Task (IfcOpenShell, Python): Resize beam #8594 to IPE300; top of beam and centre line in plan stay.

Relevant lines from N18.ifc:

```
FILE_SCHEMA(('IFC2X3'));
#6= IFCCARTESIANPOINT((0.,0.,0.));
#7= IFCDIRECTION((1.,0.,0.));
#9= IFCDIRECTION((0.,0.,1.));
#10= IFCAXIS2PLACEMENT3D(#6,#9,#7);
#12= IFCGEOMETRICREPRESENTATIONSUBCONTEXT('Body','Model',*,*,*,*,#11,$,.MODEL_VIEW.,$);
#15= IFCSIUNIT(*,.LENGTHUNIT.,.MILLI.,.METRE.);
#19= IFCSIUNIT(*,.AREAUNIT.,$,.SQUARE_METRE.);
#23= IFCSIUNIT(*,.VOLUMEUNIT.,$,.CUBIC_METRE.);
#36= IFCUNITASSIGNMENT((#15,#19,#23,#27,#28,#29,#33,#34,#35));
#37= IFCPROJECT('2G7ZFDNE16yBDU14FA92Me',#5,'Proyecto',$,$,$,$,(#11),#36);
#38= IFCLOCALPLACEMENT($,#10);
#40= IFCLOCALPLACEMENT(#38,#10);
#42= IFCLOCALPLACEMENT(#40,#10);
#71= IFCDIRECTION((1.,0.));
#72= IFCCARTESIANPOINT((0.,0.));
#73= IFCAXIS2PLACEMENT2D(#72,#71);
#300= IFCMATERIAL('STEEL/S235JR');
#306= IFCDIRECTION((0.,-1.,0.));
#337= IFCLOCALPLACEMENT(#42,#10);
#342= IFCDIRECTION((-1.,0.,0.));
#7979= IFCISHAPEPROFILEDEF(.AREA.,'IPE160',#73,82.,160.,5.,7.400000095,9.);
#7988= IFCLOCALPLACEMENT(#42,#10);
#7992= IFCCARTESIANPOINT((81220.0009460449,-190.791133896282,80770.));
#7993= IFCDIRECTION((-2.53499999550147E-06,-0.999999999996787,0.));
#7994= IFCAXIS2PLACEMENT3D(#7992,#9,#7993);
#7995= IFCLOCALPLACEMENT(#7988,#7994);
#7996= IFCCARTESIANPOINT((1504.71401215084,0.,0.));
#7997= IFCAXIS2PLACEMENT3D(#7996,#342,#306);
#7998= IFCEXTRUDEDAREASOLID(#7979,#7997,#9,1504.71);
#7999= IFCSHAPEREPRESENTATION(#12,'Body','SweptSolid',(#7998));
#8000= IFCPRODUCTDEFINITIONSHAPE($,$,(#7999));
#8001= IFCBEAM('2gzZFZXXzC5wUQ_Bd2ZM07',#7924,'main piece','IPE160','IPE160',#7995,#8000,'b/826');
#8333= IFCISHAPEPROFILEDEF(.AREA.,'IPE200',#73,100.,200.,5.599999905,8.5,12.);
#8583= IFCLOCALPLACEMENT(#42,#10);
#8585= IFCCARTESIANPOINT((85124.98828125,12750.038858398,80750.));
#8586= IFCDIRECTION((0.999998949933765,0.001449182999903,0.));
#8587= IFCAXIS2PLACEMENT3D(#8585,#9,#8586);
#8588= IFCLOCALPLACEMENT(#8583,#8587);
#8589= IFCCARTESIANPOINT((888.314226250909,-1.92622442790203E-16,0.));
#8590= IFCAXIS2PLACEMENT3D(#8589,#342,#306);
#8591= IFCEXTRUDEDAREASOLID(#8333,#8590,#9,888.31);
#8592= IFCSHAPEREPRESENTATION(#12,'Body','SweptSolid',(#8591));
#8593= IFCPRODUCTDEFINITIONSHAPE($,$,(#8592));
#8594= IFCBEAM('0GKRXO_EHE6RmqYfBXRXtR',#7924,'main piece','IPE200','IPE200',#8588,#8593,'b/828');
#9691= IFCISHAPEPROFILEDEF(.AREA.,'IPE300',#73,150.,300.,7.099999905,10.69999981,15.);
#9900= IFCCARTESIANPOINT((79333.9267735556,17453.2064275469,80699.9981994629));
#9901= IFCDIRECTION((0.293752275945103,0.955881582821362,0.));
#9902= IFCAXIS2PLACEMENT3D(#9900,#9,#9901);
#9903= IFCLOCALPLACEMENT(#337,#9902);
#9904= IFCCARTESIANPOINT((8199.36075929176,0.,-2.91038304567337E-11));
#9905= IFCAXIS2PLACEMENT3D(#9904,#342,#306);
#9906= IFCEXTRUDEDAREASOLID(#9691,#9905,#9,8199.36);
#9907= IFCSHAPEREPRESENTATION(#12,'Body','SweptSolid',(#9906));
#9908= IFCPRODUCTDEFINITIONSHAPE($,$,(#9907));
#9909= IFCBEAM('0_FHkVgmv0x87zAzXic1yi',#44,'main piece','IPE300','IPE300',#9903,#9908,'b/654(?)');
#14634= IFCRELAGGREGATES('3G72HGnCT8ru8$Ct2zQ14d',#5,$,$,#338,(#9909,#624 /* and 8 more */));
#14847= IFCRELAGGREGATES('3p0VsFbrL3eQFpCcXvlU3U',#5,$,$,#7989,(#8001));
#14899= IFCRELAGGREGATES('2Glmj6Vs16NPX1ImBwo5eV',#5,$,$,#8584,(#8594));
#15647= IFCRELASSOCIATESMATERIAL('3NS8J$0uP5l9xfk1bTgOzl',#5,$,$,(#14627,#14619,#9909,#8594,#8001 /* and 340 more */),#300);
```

```python
import ifcopenshell
import ifcopenshell.util.element
import ifcopenshell.util.representation

model = ifcopenshell.open("N18.ifc")

member = model.by_guid("0GKRXO_EHE6RmqYfBXRXtR")
source = next(p for p in model.by_type("IfcIShapeProfileDef") if p.ProfileName == "IPE300")

body = ifcopenshell.util.representation.get_representation(member, "Model", "Body")
solid = body.Items[0]
old_profile = solid.SweptArea

# Copy the section's sizes but keep this member's own profile position.
profile = ifcopenshell.util.element.copy(model, source)
# Profiles are centred, so shift by half the change in depth to hold the top.
shift = (old_profile.OverallDepth - profile.OverallDepth) / 2
x, y = old_profile.Position.Location.Coordinates
up = (0.0, 1.0)  # upwards, in the solid's own plane
location = model.createIfcCartesianPoint((x + up[0] * shift, y + up[1] * shift))
profile.Position = model.createIfcAxis2Placement2D(location, old_profile.Position.RefDirection)
solid.SweptArea = profile
if not model.get_total_inverses(old_profile):
    ifcopenshell.util.element.remove_deep2(model, old_profile)
member.Description = member.Description.replace("IPE200", "IPE300")
member.ObjectType = member.ObjectType.replace("IPE200", "IPE300")

print(solid.SweptArea)

model.write("N18_updated.ifc")
```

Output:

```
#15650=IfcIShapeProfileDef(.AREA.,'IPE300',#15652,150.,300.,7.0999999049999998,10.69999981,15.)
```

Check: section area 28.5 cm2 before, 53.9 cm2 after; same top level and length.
